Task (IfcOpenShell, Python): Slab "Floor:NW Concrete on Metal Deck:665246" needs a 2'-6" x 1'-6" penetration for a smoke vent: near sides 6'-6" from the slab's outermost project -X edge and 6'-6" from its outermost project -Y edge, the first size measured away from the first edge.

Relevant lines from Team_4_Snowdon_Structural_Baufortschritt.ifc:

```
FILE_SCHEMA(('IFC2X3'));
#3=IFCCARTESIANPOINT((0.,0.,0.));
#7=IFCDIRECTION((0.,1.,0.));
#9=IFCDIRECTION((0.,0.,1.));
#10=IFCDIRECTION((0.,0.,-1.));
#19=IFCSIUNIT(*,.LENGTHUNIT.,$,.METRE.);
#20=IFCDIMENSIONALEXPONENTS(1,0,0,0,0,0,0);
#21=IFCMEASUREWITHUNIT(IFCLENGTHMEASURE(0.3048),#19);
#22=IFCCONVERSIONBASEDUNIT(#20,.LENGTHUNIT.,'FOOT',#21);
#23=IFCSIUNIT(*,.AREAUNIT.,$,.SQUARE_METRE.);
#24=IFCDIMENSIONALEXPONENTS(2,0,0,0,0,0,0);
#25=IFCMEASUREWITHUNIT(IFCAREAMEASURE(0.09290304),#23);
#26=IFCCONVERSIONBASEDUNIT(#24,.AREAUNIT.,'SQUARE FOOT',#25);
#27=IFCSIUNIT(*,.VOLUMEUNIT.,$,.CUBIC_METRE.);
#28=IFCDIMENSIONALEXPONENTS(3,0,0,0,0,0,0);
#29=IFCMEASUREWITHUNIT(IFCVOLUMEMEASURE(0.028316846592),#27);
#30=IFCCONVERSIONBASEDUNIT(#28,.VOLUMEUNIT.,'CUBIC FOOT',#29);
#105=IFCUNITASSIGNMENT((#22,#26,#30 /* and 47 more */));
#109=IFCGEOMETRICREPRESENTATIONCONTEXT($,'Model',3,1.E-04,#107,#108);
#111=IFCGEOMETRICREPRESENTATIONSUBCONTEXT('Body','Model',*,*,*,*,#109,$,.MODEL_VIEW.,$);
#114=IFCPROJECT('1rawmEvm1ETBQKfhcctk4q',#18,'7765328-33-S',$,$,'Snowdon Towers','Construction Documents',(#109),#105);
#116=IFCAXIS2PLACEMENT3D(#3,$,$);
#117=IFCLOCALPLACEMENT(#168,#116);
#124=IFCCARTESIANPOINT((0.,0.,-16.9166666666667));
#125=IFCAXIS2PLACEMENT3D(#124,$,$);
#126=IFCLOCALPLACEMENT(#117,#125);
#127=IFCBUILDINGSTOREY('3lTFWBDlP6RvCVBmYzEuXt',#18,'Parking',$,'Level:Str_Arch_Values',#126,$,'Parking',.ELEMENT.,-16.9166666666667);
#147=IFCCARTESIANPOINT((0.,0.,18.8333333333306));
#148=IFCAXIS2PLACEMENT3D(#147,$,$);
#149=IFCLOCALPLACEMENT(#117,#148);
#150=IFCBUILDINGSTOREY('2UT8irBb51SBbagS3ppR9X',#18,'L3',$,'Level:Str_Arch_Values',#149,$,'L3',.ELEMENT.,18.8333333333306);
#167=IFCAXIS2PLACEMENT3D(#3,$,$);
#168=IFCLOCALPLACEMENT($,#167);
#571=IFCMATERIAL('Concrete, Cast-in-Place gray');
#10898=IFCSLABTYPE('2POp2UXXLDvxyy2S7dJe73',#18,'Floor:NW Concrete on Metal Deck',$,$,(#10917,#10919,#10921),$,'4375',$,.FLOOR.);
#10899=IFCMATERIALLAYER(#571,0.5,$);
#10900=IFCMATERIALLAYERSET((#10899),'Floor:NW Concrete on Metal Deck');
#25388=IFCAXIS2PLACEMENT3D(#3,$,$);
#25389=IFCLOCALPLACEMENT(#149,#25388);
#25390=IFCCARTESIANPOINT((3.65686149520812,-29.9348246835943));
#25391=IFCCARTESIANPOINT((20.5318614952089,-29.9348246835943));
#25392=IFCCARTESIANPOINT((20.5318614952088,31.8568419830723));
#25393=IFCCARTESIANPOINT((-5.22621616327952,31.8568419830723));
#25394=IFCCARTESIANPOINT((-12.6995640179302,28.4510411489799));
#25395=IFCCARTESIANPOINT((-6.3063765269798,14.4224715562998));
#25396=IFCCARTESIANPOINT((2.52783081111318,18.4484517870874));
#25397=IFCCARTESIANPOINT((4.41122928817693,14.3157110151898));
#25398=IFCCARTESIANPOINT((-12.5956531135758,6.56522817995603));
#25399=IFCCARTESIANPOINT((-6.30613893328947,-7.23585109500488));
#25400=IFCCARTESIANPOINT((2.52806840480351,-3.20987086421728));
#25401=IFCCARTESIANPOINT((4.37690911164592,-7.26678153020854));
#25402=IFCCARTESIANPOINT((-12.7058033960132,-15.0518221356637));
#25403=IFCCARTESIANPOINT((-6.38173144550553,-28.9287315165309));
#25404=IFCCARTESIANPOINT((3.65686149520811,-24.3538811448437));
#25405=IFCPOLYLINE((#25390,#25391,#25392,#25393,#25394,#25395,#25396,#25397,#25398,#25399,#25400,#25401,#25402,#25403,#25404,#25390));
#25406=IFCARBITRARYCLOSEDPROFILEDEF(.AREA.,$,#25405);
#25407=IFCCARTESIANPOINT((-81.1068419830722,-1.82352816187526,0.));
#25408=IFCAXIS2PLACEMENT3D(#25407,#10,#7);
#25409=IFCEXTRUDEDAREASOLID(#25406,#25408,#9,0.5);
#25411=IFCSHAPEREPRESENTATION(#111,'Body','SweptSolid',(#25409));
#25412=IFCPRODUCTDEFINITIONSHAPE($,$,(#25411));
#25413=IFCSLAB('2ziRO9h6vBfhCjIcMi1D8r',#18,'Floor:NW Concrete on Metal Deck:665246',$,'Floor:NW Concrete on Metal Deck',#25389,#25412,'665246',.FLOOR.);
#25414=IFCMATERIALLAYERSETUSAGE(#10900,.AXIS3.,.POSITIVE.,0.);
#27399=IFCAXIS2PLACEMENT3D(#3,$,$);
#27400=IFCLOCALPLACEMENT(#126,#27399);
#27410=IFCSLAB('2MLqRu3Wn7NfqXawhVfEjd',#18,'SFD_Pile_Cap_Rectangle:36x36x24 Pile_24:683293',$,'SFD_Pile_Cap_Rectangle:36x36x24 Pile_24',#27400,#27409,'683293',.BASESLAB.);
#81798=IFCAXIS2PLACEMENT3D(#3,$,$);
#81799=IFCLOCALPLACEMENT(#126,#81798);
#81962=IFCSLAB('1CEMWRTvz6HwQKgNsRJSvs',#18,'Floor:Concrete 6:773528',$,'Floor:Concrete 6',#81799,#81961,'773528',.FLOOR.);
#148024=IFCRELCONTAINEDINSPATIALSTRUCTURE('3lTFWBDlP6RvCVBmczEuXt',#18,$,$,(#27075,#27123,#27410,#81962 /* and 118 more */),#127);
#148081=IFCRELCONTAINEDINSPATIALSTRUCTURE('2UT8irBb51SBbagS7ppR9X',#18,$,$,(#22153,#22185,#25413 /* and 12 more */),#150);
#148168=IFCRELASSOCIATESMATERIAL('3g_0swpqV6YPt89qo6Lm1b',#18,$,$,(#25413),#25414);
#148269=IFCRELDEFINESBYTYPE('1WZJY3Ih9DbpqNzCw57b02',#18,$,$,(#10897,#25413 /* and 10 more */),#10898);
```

```python
import numpy as np
import ifcopenshell
import ifcopenshell.api.feature
import ifcopenshell.api.geometry
import ifcopenshell.api.root
import ifcopenshell.geom
import ifcopenshell.util.placement
import ifcopenshell.util.representation
import ifcopenshell.util.shape
import ifcopenshell.util.unit

model = ifcopenshell.open("Team_4_Snowdon_Structural_Baufortschritt.ifc")
unit_scale = ifcopenshell.util.unit.calculate_unit_scale(model)
settings = ifcopenshell.geom.settings()


def volume(element):
    """Net volume in cubic metres, openings subtracted."""
    shape = ifcopenshell.geom.create_shape(settings, element)
    return ifcopenshell.util.shape.get_volume(shape.geometry)


slab = model.by_guid("2ziRO9h6vBfhCjIcMi1D8r")
before = volume(slab)

# Extent in the slab's own axes, in metres. The edges named are its -X and -Y sides.
slab_shape = ifcopenshell.geom.create_shape(settings, slab)
vertices = ifcopenshell.util.shape.get_vertices(slab_shape.geometry)
x_min, y_min, bottom = vertices.min(axis=0)
top = vertices[:, 2].max()

opening = ifcopenshell.api.root.create_entity(model, ifc_class="IfcOpeningElement", name="Smoke vent opening")
context = ifcopenshell.util.representation.get_context(model, "Model", "Body", "MODEL_VIEW")
width, depth = 0.762, 0.4572
outline = [(0.0, 0.0), (width, 0.0), (width, depth), (0.0, depth), (0.0, 0.0)]
# Overshoot both faces by 50 mm so the cut is clean.
shape = ifcopenshell.api.geometry.add_slab_representation(
    model, context=context, depth=top - bottom + 0.1, polyline=outline
)
ifcopenshell.api.geometry.assign_representation(model, product=opening, representation=shape)

matrix = ifcopenshell.util.placement.get_local_placement(slab.ObjectPlacement)
matrix[:, 3] = matrix @ np.append(np.array([x_min + 1.9812, y_min + 1.9812, bottom - 0.05]) / unit_scale, 1.0)
ifcopenshell.api.geometry.edit_object_placement(model, product=opening, matrix=matrix, is_si=False)
ifcopenshell.api.feature.add_feature(model, feature=opening, element=slab)

after = volume(slab)

print(f"slab volume {before:.3f} -> {after:.3f} m3")

model.write("Team_4_Snowdon_Structural_Baufortschritt_rev.ifc")
```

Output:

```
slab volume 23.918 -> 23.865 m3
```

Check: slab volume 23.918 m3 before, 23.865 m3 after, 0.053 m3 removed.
